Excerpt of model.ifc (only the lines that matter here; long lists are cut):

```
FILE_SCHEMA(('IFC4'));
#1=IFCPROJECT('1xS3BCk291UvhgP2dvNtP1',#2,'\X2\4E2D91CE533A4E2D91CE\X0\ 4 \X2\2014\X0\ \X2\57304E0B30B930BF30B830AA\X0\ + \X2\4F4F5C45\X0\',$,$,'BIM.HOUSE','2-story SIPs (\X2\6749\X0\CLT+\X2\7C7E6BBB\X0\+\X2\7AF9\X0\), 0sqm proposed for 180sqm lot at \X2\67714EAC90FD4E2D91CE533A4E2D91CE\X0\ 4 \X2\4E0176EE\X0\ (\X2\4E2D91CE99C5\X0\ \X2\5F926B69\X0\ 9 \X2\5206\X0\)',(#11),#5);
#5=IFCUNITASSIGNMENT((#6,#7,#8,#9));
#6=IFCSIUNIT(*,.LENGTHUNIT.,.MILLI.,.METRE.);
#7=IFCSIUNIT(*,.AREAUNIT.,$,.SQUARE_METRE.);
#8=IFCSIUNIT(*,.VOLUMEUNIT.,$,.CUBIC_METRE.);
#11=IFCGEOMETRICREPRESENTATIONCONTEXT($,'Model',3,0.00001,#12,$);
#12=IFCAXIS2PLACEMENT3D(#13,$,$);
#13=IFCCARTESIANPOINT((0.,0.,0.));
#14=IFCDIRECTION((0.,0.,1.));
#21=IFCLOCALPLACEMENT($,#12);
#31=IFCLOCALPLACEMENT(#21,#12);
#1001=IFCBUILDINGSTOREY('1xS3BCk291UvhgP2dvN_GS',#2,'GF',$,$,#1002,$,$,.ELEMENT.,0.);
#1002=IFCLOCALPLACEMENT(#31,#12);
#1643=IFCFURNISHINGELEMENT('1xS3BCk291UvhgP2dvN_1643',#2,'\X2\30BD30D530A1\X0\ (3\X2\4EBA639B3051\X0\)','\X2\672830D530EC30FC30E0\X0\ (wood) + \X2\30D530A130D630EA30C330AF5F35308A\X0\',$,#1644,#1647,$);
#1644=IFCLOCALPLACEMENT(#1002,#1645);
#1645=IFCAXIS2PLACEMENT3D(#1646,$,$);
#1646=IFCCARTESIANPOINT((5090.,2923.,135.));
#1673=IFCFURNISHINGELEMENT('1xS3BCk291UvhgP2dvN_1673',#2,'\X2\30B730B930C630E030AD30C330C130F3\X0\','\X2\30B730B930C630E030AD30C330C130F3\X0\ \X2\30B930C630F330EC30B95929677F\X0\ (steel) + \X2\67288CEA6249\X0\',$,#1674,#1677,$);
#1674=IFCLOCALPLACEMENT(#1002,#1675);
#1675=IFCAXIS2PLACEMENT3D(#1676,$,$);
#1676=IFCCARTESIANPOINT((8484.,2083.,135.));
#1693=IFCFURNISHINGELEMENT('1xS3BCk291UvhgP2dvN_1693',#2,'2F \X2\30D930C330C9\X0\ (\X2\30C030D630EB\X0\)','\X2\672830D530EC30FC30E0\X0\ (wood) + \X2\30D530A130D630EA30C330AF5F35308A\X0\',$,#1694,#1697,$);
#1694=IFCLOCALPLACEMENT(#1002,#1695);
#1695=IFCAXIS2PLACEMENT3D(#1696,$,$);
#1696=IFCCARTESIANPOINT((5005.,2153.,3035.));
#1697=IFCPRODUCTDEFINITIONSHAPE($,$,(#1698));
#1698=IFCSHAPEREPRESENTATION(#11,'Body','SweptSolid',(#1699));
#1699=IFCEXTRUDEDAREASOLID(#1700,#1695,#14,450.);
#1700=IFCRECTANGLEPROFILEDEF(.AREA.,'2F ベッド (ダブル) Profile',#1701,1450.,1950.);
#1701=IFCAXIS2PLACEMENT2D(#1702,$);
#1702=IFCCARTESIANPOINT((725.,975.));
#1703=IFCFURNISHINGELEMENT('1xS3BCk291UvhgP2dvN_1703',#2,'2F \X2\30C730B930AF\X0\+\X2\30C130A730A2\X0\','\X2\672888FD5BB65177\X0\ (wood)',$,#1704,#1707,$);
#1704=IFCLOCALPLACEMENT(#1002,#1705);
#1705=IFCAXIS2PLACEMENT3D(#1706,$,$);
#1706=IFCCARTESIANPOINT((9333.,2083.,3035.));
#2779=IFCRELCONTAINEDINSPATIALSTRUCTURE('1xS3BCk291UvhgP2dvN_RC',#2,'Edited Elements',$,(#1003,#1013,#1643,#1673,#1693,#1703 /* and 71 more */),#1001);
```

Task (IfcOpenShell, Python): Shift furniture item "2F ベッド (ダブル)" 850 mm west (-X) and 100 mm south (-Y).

```python
import ifcopenshell
import ifcopenshell.api.geometry
import ifcopenshell.util.placement
import ifcopenshell.util.unit

model = ifcopenshell.open("model.ifc")
unit_scale = ifcopenshell.util.unit.calculate_unit_scale(model)

item = model.by_guid("1xS3BCk291UvhgP2dvN_1693")
matrix = ifcopenshell.util.placement.get_local_placement(item.ObjectPlacement)
matrix[0, 3] -= 0.85 / unit_scale
matrix[1, 3] -= 0.1 / unit_scale
ifcopenshell.api.geometry.edit_object_placement(model, product=item, matrix=matrix, is_si=False)

print(ifcopenshell.util.placement.get_local_placement(item.ObjectPlacement).round(3) + 0.0)

model.write("model_updated.ifc")
```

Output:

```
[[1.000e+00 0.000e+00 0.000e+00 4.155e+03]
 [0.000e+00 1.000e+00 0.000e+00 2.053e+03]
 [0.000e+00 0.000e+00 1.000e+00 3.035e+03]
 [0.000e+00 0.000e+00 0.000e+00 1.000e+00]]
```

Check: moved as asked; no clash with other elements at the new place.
